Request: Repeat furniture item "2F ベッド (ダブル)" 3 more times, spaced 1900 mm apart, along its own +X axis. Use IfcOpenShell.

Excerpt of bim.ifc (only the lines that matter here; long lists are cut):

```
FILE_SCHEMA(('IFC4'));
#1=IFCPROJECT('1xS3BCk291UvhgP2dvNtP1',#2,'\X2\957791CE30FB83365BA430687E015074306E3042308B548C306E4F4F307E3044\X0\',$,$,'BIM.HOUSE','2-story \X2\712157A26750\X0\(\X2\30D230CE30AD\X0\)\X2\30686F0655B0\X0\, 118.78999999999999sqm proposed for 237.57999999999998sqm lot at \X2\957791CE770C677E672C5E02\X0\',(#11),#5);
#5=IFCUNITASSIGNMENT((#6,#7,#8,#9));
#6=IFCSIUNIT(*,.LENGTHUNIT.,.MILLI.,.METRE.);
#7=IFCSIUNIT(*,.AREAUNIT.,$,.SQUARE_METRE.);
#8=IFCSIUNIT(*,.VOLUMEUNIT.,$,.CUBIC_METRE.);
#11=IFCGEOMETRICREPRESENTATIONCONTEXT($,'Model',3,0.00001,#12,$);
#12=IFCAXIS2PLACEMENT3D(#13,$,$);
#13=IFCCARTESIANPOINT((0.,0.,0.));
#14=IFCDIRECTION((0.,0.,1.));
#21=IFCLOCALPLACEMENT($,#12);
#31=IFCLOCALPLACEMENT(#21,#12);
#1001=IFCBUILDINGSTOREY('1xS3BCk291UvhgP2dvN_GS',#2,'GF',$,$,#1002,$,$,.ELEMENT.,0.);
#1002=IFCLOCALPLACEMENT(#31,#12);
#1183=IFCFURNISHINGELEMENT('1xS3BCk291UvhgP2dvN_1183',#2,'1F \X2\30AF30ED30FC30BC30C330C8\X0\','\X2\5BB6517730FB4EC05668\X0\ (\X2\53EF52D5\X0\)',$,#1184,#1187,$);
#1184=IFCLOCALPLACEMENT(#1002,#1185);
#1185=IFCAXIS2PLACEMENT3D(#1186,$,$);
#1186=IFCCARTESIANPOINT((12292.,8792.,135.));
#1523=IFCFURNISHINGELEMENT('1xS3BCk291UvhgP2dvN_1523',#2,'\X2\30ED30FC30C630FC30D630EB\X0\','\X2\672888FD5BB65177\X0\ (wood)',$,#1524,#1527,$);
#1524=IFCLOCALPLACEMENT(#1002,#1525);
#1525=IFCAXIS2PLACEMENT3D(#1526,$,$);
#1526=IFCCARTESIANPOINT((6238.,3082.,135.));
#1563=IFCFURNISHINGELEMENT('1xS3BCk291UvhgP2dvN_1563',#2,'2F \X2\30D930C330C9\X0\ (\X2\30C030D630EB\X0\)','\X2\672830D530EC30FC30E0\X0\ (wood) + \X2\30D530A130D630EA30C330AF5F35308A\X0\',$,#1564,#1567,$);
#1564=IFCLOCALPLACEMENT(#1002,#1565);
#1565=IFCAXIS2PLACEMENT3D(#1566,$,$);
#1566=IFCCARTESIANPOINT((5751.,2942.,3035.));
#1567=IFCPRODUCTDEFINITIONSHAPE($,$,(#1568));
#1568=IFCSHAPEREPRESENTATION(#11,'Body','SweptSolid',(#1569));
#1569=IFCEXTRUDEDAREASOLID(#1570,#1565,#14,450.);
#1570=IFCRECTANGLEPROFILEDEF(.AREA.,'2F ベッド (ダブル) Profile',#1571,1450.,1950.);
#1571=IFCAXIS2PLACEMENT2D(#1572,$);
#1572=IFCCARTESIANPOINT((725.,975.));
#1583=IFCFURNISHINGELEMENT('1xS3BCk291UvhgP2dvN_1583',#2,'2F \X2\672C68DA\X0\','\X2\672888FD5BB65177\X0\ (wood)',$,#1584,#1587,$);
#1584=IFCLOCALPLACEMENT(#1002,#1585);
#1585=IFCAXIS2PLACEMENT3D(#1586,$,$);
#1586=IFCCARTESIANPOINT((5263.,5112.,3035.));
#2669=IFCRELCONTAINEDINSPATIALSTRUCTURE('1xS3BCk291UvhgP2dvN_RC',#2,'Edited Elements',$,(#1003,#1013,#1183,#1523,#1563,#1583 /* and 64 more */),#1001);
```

```python
import ifcopenshell
import ifcopenshell.api.geometry
import ifcopenshell.api.root
import ifcopenshell.util.element
import ifcopenshell.util.placement

model = ifcopenshell.open("bim.ifc")


def reuse_history(source, copy):
    """copy_class also copies each property set's owner history, people and application; keep the originals."""
    for rel in copy.IsDefinedBy:
        if rel.is_a("IfcRelDefinesByProperties") and (history := rel.RelatingPropertyDefinition.OwnerHistory):
            rel.RelatingPropertyDefinition.OwnerHistory = source.OwnerHistory
            ifcopenshell.util.element.remove_deep2(model, history)


source = model.by_guid("1xS3BCk291UvhgP2dvN_1563")
base = ifcopenshell.util.placement.get_local_placement(source.ObjectPlacement)
step = base[:3, 0] * 1900.0

for i in range(1, 4):
    copy = ifcopenshell.api.root.copy_class(model, product=source)
    copy.Representation = ifcopenshell.util.element.copy_deep(
        model, source.Representation, exclude=["IfcGeometricRepresentationContext", "IfcRepresentationMap"]
    )
    reuse_history(source, copy)
    matrix = base.copy()
    matrix[:3, 3] += i * step
    print("added at", matrix[:3, 3].round(3) + 0.0)
    ifcopenshell.api.geometry.edit_object_placement(model, product=copy, matrix=matrix, is_si=False)

model.write("bim-out.ifc")
```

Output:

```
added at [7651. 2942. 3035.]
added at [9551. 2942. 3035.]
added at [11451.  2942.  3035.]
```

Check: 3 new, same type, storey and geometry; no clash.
